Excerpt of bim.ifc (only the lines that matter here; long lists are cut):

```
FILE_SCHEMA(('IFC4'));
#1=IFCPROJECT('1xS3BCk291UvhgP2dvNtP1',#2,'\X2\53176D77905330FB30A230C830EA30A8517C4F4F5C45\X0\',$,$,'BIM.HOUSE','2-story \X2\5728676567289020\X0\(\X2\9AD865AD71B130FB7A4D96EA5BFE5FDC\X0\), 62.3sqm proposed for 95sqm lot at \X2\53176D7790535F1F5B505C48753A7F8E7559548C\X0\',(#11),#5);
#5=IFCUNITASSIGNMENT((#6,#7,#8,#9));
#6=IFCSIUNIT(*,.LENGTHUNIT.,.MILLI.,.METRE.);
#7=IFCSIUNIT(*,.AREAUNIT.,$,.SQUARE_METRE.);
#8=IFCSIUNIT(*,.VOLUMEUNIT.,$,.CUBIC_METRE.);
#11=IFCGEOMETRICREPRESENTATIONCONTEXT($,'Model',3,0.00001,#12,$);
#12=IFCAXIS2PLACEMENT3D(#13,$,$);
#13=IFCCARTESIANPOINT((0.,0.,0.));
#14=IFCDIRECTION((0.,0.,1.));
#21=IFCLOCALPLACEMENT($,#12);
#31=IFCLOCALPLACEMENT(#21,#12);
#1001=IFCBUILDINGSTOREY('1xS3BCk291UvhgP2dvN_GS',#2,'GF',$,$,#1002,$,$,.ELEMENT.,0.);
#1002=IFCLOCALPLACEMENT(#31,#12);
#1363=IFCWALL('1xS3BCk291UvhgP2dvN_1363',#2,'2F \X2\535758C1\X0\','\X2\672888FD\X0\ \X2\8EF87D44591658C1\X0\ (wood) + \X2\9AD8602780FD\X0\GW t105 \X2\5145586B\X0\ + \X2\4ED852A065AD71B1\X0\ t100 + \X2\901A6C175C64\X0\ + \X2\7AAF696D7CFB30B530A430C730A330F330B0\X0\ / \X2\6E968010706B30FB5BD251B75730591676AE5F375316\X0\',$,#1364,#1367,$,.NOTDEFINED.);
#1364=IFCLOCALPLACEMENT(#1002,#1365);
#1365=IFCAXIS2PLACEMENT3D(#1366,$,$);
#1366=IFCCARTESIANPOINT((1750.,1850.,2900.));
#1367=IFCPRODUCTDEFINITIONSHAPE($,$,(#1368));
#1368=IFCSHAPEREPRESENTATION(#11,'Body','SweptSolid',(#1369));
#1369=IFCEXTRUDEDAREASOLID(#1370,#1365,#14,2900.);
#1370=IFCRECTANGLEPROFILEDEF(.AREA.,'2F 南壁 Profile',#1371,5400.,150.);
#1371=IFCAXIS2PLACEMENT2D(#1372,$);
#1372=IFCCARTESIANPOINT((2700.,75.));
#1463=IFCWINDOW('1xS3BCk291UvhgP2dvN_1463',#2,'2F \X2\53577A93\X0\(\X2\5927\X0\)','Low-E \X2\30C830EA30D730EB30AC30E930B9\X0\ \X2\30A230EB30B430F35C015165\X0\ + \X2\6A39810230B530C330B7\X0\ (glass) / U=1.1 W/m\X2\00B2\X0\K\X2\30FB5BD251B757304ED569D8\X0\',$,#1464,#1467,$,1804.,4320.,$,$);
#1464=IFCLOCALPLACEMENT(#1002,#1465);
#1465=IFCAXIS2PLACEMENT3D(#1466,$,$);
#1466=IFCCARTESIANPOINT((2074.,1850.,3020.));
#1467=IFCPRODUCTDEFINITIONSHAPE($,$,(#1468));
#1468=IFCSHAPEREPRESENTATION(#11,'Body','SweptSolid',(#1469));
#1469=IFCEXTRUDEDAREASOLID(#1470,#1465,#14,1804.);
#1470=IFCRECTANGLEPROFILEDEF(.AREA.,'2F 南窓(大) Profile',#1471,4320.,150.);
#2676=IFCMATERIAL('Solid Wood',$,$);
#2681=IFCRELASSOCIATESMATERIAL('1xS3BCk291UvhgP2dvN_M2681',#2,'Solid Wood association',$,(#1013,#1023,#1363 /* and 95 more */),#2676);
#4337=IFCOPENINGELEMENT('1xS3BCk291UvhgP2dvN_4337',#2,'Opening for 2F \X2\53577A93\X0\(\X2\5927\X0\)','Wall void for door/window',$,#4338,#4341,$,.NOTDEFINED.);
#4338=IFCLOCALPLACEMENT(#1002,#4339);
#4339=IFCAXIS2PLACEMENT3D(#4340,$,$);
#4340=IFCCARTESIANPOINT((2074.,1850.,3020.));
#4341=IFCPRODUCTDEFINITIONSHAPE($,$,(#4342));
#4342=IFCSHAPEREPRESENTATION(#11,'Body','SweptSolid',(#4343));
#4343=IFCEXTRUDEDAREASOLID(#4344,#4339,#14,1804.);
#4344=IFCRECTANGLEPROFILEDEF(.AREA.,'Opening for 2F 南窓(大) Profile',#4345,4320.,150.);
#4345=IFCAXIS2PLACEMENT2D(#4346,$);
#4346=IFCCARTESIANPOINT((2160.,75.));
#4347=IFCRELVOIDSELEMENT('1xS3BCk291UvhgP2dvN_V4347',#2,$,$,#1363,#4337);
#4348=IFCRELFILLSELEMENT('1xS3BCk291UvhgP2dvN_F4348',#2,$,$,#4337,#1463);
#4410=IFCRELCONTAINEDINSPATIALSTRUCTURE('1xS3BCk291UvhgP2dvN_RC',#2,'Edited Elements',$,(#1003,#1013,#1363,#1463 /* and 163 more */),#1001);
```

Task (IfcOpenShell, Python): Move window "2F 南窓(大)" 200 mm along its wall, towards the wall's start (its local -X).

```python
import ifcopenshell
import ifcopenshell.api.geometry
import ifcopenshell.util.placement
import ifcopenshell.util.unit

model = ifcopenshell.open("bim.ifc")
unit_scale = ifcopenshell.util.unit.calculate_unit_scale(model)

window = model.by_guid("1xS3BCk291UvhgP2dvN_1463")
opening = window.FillsVoids[0].RelatingOpeningElement
wall = opening.VoidsElements[0].RelatingBuildingElement

wall_matrix = ifcopenshell.util.placement.get_local_placement(wall.ObjectPlacement)
shift = wall_matrix[:3, 0] * -0.2 / unit_scale
before = ifcopenshell.util.placement.get_local_placement(window.ObjectPlacement)[:3, 3].copy()

# The window is not placed relative to its opening, so move both.
for product in (opening, window):
    matrix = ifcopenshell.util.placement.get_local_placement(product.ObjectPlacement)
    matrix[:3, 3] += shift
    ifcopenshell.api.geometry.edit_object_placement(model, product=product, matrix=matrix, is_si=False)

after = ifcopenshell.util.placement.get_local_placement(window.ObjectPlacement)[:3, 3]
print("window moved by", (after - before).round(3) + 0.0)

model.write("bim-out.ifc")
```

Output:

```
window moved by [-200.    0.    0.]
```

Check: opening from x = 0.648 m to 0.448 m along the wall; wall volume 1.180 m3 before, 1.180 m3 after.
